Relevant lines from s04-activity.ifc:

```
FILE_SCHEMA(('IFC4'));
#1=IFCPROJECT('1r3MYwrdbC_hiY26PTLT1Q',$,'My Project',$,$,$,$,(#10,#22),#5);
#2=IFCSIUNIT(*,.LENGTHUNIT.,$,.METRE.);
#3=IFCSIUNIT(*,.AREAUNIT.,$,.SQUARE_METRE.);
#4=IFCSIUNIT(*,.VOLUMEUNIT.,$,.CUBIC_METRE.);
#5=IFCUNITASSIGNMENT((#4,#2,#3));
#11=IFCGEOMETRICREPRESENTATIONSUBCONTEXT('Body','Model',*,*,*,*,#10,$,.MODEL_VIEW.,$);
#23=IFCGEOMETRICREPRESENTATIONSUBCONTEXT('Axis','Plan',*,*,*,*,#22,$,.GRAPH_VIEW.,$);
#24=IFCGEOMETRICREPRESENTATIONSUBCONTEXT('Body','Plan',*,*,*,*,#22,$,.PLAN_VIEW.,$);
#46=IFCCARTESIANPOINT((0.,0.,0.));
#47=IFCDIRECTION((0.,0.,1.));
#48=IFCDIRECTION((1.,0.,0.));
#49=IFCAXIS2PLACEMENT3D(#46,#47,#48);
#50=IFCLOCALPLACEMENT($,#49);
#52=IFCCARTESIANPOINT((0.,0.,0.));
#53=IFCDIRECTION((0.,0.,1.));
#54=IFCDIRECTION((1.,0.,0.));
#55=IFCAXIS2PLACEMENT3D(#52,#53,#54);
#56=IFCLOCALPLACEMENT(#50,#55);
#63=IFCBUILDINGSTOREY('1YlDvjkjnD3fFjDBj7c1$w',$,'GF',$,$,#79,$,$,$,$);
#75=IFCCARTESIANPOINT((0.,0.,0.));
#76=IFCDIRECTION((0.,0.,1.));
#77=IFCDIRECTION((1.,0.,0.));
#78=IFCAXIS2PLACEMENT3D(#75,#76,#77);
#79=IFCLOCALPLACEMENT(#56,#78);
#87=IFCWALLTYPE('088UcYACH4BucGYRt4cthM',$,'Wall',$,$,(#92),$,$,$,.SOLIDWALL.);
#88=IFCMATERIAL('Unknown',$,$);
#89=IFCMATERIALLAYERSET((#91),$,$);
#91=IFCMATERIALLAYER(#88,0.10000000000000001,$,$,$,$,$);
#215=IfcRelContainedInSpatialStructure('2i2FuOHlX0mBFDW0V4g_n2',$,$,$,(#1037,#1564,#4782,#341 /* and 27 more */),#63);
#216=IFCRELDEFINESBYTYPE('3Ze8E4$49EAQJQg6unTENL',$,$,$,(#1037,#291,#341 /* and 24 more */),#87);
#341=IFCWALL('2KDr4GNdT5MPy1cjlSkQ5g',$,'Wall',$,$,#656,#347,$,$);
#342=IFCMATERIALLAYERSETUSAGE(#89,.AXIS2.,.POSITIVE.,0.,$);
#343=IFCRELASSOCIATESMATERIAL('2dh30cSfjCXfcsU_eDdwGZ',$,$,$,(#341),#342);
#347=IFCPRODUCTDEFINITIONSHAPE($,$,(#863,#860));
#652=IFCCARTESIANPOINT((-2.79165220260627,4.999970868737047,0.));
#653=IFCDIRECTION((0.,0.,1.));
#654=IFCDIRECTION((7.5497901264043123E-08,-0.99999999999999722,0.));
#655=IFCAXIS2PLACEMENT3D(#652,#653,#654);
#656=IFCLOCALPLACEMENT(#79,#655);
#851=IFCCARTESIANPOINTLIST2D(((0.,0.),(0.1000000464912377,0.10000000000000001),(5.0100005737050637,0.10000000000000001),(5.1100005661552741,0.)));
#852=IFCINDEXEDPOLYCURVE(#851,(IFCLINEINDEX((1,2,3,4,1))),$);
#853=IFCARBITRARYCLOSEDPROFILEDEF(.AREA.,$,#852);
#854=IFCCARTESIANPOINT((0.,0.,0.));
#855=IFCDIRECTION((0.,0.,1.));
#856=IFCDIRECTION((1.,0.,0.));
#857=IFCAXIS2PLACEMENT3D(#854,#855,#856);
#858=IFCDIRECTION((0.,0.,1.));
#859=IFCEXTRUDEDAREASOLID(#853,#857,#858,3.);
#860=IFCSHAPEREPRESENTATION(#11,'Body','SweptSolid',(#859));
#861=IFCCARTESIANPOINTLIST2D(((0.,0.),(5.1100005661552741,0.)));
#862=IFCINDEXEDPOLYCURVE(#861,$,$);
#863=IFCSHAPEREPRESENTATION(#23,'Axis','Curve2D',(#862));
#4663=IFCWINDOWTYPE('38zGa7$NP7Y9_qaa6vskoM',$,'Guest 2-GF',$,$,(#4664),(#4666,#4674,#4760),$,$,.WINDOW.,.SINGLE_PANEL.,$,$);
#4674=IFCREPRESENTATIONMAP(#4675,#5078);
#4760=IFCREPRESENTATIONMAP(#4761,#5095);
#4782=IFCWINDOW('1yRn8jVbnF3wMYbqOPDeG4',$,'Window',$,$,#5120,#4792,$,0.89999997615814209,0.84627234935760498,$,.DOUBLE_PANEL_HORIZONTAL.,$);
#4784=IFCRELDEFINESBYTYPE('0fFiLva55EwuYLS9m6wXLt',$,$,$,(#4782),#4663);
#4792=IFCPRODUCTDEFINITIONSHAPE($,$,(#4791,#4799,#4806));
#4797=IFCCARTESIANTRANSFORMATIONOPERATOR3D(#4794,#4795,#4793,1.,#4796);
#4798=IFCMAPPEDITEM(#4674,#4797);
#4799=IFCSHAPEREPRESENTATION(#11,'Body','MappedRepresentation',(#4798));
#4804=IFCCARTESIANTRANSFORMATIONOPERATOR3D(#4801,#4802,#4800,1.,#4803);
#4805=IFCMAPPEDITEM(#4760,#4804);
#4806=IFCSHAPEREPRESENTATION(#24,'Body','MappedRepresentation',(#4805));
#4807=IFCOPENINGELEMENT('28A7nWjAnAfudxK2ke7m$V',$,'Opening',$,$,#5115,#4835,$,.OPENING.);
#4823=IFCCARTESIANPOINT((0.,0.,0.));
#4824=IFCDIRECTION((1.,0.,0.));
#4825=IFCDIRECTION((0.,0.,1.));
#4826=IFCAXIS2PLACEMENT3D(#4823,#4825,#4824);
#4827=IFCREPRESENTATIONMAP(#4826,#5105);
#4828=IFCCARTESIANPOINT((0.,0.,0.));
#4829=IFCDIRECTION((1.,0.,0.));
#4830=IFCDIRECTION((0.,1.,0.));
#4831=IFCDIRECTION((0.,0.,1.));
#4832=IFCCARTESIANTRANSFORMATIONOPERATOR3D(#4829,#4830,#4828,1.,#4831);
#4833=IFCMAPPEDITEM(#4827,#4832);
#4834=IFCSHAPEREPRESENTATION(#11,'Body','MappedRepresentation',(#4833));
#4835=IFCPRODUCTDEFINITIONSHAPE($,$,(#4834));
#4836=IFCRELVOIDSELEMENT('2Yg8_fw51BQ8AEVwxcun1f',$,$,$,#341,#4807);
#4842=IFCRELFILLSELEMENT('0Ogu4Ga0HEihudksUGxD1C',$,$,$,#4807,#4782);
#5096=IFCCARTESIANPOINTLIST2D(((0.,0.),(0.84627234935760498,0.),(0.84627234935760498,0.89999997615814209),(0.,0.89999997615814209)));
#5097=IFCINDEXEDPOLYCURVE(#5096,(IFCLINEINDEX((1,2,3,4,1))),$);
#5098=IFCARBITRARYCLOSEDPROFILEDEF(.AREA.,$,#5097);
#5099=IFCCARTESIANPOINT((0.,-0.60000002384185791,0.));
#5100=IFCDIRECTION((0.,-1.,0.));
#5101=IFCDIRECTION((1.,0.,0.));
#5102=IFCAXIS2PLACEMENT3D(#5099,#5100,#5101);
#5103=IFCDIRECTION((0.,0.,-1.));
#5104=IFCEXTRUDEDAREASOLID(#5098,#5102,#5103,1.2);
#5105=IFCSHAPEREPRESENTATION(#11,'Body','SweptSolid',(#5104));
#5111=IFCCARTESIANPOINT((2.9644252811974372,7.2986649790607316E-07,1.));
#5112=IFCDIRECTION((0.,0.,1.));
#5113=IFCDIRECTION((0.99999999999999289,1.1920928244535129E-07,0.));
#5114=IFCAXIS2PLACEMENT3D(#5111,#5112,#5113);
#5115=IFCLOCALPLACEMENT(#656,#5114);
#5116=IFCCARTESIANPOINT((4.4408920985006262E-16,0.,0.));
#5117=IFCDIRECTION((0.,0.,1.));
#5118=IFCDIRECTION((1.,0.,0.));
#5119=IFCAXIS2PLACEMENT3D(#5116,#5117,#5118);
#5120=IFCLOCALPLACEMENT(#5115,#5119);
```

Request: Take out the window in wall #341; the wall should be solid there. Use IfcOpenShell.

```python
import ifcopenshell
import ifcopenshell.api.feature
import ifcopenshell.api.root
import ifcopenshell.geom
import ifcopenshell.util.shape

model = ifcopenshell.open("s04-activity.ifc")
settings = ifcopenshell.geom.settings()


def volume(element):
    """Net volume in cubic metres, openings subtracted."""
    shape = ifcopenshell.geom.create_shape(settings, element)
    return ifcopenshell.util.shape.get_volume(shape.geometry)


window = model.by_guid("1yRn8jVbnF3wMYbqOPDeG4")
opening = window.FillsVoids[0].RelatingOpeningElement
wall = opening.VoidsElements[0].RelatingBuildingElement
before = volume(wall)

ifcopenshell.api.root.remove_product(model, product=window)
ifcopenshell.api.feature.remove_feature(model, feature=opening)

after = volume(wall)

print(f"wall volume {before:.3f} -> {after:.3f} m3")

model.write("s04-activity_updated.ifc")
```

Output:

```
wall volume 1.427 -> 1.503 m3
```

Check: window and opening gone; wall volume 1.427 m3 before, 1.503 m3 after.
